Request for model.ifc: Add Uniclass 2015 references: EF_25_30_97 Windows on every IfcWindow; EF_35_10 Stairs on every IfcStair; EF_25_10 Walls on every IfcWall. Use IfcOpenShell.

First a look at what the model holds.

```python
import ifcopenshell

model = ifcopenshell.open("model.ifc")
print(model.schema)
print("classifications:", [c.Name for c in model.by_type("IfcClassification")])
for ifc_class in ("IfcDoor", "IfcRoof", "IfcStair", "IfcWall", "IfcWindow"):
    print(ifc_class, len(model.by_type(ifc_class)))
```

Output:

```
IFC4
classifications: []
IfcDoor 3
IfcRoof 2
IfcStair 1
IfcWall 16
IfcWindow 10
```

```python
import ifcopenshell
import ifcopenshell.api.classification

model = ifcopenshell.open("model.ifc")

system = ifcopenshell.api.classification.add_classification(model, classification="Uniclass 2015")

codes = {
    "IfcWindow": ("EF_25_30_97", "Windows"),
    "IfcStair": ("EF_35_10", "Stairs"),
    "IfcWall": ("EF_25_10", "Walls"),
}
for ifc_class, (code, name) in codes.items():
    products = model.by_type(ifc_class)
    ifcopenshell.api.classification.add_reference(
        model, products=products, classification=system, identification=code, name=name
    )
    print(code, len(products))

model.write("model_updated.ifc")
```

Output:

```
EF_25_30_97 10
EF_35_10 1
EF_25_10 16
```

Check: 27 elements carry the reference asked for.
